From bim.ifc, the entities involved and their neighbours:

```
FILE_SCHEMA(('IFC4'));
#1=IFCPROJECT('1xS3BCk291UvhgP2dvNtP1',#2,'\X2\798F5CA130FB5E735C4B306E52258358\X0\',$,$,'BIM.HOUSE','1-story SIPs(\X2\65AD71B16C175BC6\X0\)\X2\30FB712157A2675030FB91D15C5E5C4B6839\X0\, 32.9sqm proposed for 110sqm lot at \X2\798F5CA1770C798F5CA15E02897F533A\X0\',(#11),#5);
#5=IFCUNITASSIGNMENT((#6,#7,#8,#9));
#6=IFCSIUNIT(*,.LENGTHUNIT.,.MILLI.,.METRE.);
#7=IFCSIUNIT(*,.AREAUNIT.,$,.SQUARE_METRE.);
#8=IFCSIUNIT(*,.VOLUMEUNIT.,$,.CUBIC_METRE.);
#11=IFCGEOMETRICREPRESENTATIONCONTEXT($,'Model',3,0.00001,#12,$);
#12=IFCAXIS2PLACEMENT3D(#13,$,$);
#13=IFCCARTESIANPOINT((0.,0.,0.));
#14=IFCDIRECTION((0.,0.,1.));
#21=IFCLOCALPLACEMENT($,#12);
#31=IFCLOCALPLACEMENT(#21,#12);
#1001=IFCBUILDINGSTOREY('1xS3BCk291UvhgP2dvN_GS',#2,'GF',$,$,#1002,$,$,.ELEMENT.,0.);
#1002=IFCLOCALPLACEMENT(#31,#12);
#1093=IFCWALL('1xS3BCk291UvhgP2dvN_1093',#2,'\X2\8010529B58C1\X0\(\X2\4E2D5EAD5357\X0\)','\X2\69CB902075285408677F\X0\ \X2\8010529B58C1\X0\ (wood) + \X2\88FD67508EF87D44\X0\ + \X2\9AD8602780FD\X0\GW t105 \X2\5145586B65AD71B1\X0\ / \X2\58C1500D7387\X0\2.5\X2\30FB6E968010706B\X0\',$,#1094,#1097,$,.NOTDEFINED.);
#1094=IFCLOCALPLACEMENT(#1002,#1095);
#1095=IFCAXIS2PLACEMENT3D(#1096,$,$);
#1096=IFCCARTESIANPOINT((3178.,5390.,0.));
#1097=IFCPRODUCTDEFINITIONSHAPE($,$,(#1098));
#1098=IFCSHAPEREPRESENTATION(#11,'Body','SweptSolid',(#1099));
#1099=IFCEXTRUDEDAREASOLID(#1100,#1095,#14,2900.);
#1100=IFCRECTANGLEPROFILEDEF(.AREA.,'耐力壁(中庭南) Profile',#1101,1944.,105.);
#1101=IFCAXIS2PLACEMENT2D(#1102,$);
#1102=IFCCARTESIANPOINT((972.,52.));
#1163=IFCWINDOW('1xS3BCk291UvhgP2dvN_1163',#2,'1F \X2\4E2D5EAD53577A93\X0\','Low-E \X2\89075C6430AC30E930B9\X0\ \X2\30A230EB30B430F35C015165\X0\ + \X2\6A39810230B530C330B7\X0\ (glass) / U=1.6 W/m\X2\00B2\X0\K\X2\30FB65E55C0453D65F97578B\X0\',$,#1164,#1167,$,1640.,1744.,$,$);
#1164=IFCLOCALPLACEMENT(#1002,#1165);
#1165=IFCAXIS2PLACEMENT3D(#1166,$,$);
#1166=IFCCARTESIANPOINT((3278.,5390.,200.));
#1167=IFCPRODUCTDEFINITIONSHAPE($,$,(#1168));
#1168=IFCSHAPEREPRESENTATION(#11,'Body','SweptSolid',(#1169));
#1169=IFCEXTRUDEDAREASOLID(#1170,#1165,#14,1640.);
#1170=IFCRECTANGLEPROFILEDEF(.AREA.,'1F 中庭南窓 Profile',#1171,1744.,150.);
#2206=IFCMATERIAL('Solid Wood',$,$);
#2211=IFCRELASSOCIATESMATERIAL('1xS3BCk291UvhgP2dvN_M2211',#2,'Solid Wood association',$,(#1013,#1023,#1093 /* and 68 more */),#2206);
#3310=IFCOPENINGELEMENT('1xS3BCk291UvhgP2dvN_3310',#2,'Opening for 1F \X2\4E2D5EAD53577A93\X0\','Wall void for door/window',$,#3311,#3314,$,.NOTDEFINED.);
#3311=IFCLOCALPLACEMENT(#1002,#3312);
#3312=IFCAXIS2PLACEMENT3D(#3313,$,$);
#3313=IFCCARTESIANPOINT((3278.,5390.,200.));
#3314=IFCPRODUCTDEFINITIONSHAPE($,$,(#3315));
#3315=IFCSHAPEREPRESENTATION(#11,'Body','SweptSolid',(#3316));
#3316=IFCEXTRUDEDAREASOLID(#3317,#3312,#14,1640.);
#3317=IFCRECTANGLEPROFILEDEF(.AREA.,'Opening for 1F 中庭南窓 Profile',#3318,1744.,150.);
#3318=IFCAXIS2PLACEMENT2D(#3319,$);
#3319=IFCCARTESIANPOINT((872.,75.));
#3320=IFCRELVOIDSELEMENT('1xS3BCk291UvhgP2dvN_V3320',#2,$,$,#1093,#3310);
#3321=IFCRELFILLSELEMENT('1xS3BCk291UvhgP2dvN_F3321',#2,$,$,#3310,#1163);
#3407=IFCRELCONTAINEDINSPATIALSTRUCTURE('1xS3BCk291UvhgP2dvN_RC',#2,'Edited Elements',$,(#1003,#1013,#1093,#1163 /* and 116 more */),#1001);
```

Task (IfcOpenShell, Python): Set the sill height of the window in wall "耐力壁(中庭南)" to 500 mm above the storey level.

```python
import numpy as np
import ifcopenshell
import ifcopenshell.api.geometry
import ifcopenshell.geom
import ifcopenshell.util.element
import ifcopenshell.util.placement
import ifcopenshell.util.shape
import ifcopenshell.util.unit

model = ifcopenshell.open("bim.ifc")
unit_scale = ifcopenshell.util.unit.calculate_unit_scale(model)

window = model.by_guid("1xS3BCk291UvhgP2dvN_1163")
opening = window.FillsVoids[0].RelatingOpeningElement
storey = ifcopenshell.util.element.get_container(window, ifc_class="IfcBuildingStorey")
level = ifcopenshell.util.placement.get_local_placement(storey.ObjectPlacement)[2, 3]

# The opening's origin need not be at the sill, so measure its lowest point.
shape = ifcopenshell.geom.create_shape(ifcopenshell.geom.settings(), opening)
bottom = ifcopenshell.util.shape.get_shape_bottom_elevation(shape, shape.geometry) / unit_scale
dz = level + 500.0 - bottom

shift = np.array([0.0, 0.0, dz])
# The window is not placed relative to its opening, so move both.
for product in (opening, window):
    matrix = ifcopenshell.util.placement.get_local_placement(product.ObjectPlacement)
    matrix[:3, 3] += shift
    ifcopenshell.api.geometry.edit_object_placement(model, product=product, matrix=matrix, is_si=False)

print(f"moved by {dz * unit_scale:+.3f} m")

model.write("bim_updated.ifc")
```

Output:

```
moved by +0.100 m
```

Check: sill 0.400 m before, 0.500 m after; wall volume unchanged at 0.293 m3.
